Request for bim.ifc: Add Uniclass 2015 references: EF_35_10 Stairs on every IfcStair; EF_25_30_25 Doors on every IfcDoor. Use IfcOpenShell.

First a look at what the model holds.

```python
import ifcopenshell

model = ifcopenshell.open("bim.ifc")
print(model.schema)
print("classifications:", [c.Name for c in model.by_type("IfcClassification")])
for ifc_class in ("IfcDoor", "IfcRoof", "IfcStair", "IfcWall", "IfcWindow"):
    print(ifc_class, len(model.by_type(ifc_class)))
```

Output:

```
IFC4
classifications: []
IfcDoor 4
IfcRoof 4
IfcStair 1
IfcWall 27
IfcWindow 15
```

```python
import ifcopenshell
import ifcopenshell.api.classification

model = ifcopenshell.open("bim.ifc")

system = ifcopenshell.api.classification.add_classification(model, classification="Uniclass 2015")

codes = {
    "IfcStair": ("EF_35_10", "Stairs"),
    "IfcDoor": ("EF_25_30_25", "Doors"),
}
for ifc_class, (code, name) in codes.items():
    products = model.by_type(ifc_class)
    ifcopenshell.api.classification.add_reference(
        model, products=products, classification=system, identification=code, name=name
    )
    print(code, len(products))

model.write("bim-out.ifc")
```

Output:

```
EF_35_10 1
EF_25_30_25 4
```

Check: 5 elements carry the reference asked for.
